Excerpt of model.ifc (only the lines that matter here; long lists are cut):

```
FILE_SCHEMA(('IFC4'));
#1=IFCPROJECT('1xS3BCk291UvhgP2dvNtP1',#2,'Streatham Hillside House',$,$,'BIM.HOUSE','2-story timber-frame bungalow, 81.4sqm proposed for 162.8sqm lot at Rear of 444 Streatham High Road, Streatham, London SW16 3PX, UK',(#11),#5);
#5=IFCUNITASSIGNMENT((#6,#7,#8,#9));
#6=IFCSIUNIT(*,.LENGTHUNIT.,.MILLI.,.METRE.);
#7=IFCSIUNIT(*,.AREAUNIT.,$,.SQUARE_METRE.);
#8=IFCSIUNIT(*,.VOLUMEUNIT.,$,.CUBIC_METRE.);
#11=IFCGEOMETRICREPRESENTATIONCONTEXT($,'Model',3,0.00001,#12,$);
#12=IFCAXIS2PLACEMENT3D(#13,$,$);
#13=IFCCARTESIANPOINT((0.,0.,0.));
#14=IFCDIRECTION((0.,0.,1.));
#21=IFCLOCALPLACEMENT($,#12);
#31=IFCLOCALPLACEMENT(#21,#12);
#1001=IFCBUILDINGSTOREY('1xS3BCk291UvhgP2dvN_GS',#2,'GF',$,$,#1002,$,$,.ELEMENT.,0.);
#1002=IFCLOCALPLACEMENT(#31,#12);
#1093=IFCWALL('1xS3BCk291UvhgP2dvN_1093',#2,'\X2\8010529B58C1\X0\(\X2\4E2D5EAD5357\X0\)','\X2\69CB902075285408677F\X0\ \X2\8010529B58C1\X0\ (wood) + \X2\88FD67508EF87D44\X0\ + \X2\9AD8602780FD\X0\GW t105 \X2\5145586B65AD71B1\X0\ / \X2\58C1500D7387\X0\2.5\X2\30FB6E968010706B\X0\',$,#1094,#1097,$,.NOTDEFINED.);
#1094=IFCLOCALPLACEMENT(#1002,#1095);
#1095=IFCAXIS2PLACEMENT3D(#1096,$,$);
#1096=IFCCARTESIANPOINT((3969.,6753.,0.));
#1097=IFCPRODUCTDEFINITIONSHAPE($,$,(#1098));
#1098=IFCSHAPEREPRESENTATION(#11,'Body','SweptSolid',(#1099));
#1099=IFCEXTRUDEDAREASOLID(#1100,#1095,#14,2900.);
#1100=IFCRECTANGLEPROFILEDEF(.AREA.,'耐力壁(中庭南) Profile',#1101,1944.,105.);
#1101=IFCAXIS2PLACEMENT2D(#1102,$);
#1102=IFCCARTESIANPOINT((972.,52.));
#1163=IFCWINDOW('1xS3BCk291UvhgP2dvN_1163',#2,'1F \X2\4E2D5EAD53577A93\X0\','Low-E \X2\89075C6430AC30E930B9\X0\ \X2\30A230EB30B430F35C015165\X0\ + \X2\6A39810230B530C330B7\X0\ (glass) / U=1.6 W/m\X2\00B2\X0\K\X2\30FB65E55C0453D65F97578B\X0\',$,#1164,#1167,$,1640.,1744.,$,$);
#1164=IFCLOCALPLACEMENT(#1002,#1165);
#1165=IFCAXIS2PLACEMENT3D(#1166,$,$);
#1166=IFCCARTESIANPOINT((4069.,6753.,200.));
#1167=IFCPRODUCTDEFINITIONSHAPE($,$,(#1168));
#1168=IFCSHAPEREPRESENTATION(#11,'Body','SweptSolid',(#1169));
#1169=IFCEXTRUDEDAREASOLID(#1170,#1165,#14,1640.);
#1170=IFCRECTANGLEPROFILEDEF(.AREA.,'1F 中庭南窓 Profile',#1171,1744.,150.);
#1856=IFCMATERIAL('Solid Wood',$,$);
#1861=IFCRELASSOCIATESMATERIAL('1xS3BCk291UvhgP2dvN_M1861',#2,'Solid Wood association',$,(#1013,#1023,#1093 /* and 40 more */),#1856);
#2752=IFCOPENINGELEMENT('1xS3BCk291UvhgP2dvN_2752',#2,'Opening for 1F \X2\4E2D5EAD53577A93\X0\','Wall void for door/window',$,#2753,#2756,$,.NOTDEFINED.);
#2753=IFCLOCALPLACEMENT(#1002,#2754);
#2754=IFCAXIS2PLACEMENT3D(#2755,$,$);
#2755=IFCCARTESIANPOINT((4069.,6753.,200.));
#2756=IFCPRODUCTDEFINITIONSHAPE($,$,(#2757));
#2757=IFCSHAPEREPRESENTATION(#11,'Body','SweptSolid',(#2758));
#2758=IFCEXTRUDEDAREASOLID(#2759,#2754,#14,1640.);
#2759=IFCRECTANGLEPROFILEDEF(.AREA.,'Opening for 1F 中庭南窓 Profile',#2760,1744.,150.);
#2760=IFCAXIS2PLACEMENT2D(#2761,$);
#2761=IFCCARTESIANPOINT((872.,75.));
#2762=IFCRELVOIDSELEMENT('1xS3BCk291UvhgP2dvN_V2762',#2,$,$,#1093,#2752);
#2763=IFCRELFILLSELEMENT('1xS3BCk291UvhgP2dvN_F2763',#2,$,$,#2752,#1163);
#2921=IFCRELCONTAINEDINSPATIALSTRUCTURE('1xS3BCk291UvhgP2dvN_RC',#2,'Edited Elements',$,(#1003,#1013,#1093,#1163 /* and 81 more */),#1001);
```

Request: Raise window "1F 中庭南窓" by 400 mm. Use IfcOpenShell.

```python
import numpy as np
import ifcopenshell
import ifcopenshell.api.geometry
import ifcopenshell.util.placement
import ifcopenshell.util.unit

model = ifcopenshell.open("model.ifc")
unit_scale = ifcopenshell.util.unit.calculate_unit_scale(model)

window = model.by_guid("1xS3BCk291UvhgP2dvN_1163")
opening = window.FillsVoids[0].RelatingOpeningElement
dz = 400.0

shift = np.array([0.0, 0.0, dz])
# The window is not placed relative to its opening, so move both.
for product in (opening, window):
    matrix = ifcopenshell.util.placement.get_local_placement(product.ObjectPlacement)
    matrix[:3, 3] += shift
    ifcopenshell.api.geometry.edit_object_placement(model, product=product, matrix=matrix, is_si=False)

print(f"moved by {dz * unit_scale:+.3f} m")

model.write("model_edited.ifc")
```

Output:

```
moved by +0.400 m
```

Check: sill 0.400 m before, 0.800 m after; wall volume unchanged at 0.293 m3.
